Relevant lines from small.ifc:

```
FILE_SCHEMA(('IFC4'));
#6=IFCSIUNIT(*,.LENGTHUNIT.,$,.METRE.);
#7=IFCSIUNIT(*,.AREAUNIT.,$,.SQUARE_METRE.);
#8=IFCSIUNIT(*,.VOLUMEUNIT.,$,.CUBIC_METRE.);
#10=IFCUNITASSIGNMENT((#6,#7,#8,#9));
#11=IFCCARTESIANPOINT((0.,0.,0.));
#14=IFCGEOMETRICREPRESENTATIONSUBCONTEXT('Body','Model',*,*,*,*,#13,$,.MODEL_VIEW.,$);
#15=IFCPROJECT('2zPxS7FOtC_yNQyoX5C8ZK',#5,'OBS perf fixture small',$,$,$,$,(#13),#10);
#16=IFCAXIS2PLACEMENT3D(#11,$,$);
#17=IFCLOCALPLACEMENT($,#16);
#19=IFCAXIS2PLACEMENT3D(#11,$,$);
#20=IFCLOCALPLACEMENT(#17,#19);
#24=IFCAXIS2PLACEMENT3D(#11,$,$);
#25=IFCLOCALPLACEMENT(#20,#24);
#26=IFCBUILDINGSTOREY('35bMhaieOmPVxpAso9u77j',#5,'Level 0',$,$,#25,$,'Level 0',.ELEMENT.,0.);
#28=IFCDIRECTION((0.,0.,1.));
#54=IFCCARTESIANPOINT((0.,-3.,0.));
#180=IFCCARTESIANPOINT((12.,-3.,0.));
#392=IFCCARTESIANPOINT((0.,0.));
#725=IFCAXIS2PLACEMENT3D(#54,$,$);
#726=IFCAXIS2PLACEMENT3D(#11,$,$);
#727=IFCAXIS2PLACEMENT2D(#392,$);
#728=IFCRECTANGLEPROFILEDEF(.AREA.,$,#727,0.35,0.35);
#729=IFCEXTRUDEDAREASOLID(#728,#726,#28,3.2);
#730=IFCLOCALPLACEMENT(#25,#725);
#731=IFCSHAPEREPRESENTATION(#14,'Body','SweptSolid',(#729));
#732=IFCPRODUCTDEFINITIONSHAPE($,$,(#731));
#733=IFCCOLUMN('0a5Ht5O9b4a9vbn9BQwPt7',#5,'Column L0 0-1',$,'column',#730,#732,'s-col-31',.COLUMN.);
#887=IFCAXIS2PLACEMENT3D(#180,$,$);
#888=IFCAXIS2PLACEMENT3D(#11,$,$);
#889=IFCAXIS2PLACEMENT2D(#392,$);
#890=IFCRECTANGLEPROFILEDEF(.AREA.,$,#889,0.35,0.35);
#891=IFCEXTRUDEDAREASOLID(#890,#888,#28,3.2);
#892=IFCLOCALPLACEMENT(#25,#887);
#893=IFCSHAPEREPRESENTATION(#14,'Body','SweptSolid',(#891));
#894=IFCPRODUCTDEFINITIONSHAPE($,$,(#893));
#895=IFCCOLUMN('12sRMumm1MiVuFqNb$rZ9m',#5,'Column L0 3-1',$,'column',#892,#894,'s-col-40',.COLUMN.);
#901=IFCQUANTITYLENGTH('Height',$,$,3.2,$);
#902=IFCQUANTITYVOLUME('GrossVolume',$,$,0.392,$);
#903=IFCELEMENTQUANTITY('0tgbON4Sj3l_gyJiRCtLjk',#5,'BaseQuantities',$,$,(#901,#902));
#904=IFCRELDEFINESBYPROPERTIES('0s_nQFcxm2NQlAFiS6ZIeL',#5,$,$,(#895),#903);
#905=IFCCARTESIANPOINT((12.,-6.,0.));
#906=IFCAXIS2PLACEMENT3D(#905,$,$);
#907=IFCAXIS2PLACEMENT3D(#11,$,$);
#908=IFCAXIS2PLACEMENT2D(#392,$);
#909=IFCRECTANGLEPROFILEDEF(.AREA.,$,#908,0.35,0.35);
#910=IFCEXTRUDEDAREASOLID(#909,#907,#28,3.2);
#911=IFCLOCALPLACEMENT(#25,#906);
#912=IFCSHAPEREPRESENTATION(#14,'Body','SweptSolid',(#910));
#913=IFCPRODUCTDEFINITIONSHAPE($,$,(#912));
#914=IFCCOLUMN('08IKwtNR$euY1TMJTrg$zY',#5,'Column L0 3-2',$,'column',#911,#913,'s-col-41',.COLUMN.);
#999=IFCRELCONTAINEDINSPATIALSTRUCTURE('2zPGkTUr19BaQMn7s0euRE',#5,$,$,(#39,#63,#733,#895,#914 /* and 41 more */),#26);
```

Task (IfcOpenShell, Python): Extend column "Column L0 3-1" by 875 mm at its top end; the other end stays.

```python
import ifcopenshell
import ifcopenshell.api.pset
import ifcopenshell.util.element
import ifcopenshell.util.representation

model = ifcopenshell.open("small.ifc")

member = model.by_guid("12sRMumm1MiVuFqNb$rZ9m")
change = 0.875

# The extrusion runs towards the end named, so only its depth changes.
body = ifcopenshell.util.representation.get_representation(member, "Model", "Body")
solid = body.Items[0]
old_length = solid.Depth
solid.Depth += change

# Update the stored length and volume.
qto = model.by_id(ifcopenshell.util.element.get_pset(member, "BaseQuantities", should_inherit=False)["id"])
ifcopenshell.api.pset.edit_qto(model, qto=qto, properties={
    "Height": solid.Depth,
    "GrossVolume": ifcopenshell.util.element.get_pset(member, "BaseQuantities", "GrossVolume") * solid.Depth / old_length,
})

print(f"length {old_length:g} -> {solid.Depth:g}")

model.write("small-out.ifc")
```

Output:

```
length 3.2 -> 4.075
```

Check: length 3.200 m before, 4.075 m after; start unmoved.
